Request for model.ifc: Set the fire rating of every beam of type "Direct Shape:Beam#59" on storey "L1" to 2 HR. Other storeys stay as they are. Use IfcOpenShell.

First a look at what the model holds.

```python
import ifcopenshell
import ifcopenshell.util.element

model = ifcopenshell.open("model.ifc")
print(model.schema)
storey = next(s for s in model.by_type("IfcBuildingStorey") if s.Name == "L1")
beams = [e for e in ifcopenshell.util.element.get_decomposition(storey) if e.is_a("IfcBeam")]
seen = {}
for e in beams:
    element_type = ifcopenshell.util.element.get_type(e)
    key = (element_type.Name if element_type != e and element_type else None, ifcopenshell.util.element.get_pset(e, "Pset_BeamCommon", "FireRating"))
    seen[key] = seen.get(key, 0) + 1
for (name, value), count in sorted(seen.items(), key=str):
    print(count, "x", name, "|", value)
```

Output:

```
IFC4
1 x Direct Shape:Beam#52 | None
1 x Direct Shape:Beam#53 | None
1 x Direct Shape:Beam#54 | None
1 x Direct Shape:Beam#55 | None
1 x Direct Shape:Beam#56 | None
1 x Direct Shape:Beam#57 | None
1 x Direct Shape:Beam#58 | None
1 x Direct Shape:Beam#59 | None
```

```python
import ifcopenshell
import ifcopenshell.api.pset
import ifcopenshell.util.element

model = ifcopenshell.open("model.ifc")

storey = next(s for s in model.by_type("IfcBuildingStorey") if s.Name == "L1")
beams = [e for e in ifcopenshell.util.element.get_decomposition(storey) if e.is_a("IfcBeam")]

count = 0
for e in beams:
    element_type = ifcopenshell.util.element.get_type(e)
    if element_type in (None, e) or element_type.Name != "Direct Shape:Beam#59":
        continue
    # add_pset returns the element's existing set when there is one.
    pset = ifcopenshell.api.pset.add_pset(model, product=e, name="Pset_BeamCommon")
    ifcopenshell.api.pset.edit_pset(model, pset=pset, properties={"FireRating": "2 HR"})
    count += 1

print(count, "beams updated")

model.write("model_edited.ifc")
```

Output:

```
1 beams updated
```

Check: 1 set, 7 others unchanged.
